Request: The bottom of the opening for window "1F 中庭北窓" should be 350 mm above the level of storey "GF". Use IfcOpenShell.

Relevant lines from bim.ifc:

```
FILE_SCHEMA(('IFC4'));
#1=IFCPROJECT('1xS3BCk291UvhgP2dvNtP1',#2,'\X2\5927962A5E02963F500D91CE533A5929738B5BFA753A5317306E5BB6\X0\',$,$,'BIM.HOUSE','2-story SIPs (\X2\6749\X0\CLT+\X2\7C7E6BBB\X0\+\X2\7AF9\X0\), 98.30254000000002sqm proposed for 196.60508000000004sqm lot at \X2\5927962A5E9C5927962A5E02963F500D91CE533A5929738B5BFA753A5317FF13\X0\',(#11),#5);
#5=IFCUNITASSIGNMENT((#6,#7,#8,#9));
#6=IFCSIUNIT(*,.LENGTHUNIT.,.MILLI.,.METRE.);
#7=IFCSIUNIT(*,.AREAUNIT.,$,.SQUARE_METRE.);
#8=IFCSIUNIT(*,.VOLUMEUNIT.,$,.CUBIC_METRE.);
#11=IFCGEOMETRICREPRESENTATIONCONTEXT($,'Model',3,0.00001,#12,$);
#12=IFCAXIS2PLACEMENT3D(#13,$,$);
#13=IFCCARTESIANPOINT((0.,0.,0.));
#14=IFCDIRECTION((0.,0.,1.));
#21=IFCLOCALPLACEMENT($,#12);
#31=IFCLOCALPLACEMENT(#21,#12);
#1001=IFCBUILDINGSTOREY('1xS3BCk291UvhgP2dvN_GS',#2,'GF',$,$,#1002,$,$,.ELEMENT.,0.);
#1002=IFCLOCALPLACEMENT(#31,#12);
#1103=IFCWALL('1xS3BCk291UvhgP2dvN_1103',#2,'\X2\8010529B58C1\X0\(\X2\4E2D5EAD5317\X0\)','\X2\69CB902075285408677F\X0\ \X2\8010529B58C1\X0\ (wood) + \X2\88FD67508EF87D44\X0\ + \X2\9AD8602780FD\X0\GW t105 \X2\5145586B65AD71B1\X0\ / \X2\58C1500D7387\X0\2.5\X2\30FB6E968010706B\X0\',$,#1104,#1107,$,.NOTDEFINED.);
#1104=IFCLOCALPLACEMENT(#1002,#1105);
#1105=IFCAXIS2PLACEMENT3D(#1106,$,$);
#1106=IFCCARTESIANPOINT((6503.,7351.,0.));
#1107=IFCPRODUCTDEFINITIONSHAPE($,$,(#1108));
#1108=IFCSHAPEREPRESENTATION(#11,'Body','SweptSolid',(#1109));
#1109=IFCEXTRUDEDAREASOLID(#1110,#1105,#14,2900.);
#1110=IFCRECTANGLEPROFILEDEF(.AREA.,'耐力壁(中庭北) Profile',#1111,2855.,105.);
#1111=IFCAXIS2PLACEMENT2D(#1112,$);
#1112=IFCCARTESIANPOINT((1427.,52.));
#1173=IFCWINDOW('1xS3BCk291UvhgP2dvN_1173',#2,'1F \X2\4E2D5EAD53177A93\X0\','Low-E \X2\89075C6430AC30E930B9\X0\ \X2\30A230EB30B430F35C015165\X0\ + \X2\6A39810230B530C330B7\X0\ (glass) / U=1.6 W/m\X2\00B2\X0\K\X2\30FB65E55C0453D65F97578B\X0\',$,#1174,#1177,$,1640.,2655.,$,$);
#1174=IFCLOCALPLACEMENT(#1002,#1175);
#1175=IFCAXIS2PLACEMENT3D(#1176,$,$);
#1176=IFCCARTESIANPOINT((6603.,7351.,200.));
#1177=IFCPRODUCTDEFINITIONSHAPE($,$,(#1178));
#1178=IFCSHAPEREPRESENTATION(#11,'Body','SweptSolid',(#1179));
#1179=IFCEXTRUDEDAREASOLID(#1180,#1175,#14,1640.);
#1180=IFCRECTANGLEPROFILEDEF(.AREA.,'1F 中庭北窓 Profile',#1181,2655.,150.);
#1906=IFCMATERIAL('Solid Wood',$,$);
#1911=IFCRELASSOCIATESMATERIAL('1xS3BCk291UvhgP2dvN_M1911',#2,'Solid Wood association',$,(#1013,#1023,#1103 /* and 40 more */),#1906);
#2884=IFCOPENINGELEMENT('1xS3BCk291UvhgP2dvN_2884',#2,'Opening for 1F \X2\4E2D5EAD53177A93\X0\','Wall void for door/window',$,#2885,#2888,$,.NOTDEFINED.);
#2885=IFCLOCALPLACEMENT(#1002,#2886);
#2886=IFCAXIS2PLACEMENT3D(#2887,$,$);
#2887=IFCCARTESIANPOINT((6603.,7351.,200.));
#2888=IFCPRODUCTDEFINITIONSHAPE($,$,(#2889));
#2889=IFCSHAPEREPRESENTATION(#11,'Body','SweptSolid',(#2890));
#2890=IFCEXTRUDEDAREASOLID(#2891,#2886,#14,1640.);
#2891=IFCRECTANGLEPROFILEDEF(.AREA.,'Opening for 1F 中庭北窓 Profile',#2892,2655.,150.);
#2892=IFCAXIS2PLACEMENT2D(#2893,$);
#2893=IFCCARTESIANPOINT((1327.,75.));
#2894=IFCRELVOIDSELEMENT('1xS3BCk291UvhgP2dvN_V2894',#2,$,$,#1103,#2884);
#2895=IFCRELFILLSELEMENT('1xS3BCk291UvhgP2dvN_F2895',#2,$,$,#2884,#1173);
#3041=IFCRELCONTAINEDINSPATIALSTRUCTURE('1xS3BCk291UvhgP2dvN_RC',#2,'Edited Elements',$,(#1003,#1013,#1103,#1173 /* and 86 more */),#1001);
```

```python
import numpy as np
import ifcopenshell
import ifcopenshell.api.geometry
import ifcopenshell.geom
import ifcopenshell.util.element
import ifcopenshell.util.placement
import ifcopenshell.util.shape
import ifcopenshell.util.unit

model = ifcopenshell.open("bim.ifc")
unit_scale = ifcopenshell.util.unit.calculate_unit_scale(model)

window = model.by_guid("1xS3BCk291UvhgP2dvN_1173")
opening = window.FillsVoids[0].RelatingOpeningElement
storey = ifcopenshell.util.element.get_container(window, ifc_class="IfcBuildingStorey")
level = ifcopenshell.util.placement.get_local_placement(storey.ObjectPlacement)[2, 3]

# The opening's origin need not be at the sill, so measure its lowest point.
shape = ifcopenshell.geom.create_shape(ifcopenshell.geom.settings(), opening)
bottom = ifcopenshell.util.shape.get_shape_bottom_elevation(shape, shape.geometry) / unit_scale
dz = level + 350.0 - bottom

shift = np.array([0.0, 0.0, dz])
# The window is not placed relative to its opening, so move both.
for product in (opening, window):
    matrix = ifcopenshell.util.placement.get_local_placement(product.ObjectPlacement)
    matrix[:3, 3] += shift
    ifcopenshell.api.geometry.edit_object_placement(model, product=product, matrix=matrix, is_si=False)

print(f"moved by {dz * unit_scale:+.3f} m")

model.write("bim_v2.ifc")
```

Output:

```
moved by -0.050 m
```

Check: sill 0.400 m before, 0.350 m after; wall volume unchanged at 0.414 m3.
